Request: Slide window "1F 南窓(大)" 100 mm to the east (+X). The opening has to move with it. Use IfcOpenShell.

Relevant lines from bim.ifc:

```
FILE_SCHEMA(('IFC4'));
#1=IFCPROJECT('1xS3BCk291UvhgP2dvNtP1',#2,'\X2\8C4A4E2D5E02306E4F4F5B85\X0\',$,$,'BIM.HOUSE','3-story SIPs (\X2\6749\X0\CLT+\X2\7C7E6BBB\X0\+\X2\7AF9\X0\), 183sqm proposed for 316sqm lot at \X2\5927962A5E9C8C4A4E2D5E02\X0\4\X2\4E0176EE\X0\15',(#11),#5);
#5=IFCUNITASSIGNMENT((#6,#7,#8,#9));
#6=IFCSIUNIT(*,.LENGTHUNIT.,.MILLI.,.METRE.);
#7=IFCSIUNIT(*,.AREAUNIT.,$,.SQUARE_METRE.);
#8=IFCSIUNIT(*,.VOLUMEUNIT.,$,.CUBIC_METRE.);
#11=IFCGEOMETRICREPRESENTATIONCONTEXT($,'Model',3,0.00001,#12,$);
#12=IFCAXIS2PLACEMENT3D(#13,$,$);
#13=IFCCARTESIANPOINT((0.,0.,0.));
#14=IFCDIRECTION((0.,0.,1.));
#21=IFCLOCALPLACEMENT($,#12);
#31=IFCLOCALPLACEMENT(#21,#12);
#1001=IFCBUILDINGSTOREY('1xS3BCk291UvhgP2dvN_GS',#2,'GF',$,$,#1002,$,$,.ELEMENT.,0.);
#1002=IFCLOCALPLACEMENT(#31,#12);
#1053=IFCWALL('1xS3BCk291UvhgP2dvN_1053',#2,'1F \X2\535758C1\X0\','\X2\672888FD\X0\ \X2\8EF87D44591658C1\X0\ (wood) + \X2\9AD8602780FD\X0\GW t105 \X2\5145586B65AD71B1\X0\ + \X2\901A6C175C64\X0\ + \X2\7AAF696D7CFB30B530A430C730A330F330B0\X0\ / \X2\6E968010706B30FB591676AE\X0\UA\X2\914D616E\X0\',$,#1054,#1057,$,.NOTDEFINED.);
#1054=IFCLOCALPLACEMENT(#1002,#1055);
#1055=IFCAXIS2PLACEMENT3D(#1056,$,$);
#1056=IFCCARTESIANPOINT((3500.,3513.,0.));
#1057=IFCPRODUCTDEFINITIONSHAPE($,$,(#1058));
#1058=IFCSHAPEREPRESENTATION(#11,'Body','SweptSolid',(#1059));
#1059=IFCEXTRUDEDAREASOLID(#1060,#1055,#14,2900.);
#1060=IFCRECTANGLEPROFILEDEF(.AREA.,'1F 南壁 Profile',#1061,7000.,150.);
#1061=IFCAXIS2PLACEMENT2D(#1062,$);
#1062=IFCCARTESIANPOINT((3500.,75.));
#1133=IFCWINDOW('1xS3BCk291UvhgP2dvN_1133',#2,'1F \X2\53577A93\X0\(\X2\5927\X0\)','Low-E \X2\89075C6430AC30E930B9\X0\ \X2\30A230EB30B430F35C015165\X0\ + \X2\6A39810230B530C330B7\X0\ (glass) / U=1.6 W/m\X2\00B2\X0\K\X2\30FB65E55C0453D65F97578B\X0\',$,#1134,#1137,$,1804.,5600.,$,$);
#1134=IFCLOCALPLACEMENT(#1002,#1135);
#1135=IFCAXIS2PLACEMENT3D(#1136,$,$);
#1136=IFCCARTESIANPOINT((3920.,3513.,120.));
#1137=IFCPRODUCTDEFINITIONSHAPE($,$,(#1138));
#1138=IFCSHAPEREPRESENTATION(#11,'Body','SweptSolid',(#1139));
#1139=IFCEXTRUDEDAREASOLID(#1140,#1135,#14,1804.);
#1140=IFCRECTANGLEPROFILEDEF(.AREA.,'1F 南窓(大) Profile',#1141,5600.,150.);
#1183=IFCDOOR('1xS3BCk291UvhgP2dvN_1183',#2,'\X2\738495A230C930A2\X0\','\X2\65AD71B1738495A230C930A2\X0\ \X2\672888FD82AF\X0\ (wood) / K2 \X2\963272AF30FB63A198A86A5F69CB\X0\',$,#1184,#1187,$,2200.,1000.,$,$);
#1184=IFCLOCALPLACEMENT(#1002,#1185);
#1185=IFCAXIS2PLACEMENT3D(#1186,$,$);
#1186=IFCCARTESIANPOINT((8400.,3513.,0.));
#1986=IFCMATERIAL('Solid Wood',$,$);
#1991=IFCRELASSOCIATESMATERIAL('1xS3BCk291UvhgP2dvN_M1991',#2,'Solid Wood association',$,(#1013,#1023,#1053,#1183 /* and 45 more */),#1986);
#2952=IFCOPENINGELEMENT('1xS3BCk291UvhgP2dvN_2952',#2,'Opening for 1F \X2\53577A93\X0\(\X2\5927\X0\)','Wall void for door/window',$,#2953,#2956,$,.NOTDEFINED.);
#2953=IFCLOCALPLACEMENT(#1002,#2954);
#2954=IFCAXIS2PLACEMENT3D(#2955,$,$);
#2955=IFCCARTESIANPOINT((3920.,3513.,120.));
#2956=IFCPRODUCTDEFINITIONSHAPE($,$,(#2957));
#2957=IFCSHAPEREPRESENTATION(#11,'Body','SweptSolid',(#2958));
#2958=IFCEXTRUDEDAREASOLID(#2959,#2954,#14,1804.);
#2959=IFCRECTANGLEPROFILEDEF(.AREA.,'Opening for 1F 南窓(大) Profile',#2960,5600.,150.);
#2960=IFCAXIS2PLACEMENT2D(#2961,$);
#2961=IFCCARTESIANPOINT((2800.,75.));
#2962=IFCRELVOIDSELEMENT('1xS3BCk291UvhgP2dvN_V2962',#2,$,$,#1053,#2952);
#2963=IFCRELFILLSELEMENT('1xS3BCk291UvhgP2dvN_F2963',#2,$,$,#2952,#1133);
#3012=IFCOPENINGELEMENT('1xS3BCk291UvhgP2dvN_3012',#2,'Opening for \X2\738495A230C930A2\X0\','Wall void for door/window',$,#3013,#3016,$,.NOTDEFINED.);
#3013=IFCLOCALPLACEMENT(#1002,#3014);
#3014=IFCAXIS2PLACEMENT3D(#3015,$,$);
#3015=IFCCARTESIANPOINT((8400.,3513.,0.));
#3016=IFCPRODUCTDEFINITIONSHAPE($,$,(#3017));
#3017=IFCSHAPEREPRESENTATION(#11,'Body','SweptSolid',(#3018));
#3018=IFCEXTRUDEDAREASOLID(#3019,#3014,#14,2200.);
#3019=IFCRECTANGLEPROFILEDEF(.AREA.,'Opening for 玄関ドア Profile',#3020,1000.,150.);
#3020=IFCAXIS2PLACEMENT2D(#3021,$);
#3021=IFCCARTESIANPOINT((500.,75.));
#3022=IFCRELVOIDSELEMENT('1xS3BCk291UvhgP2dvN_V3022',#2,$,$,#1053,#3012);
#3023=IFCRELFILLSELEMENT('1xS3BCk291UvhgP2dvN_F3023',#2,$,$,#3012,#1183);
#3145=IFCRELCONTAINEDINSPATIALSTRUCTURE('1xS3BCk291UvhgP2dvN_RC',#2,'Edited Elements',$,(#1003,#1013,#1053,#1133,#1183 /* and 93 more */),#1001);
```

```python
import ifcopenshell
import ifcopenshell.api.geometry
import ifcopenshell.util.placement
import ifcopenshell.util.unit

model = ifcopenshell.open("bim.ifc")
unit_scale = ifcopenshell.util.unit.calculate_unit_scale(model)

window = model.by_guid("1xS3BCk291UvhgP2dvN_1133")
opening = window.FillsVoids[0].RelatingOpeningElement
wall = opening.VoidsElements[0].RelatingBuildingElement

wall_matrix = ifcopenshell.util.placement.get_local_placement(wall.ObjectPlacement)
shift = wall_matrix[:3, 0] * 0.1 / unit_scale
before = ifcopenshell.util.placement.get_local_placement(window.ObjectPlacement)[:3, 3].copy()

# The window is not placed relative to its opening, so move both.
for product in (opening, window):
    matrix = ifcopenshell.util.placement.get_local_placement(product.ObjectPlacement)
    matrix[:3, 3] += shift
    ifcopenshell.api.geometry.edit_object_placement(model, product=product, matrix=matrix, is_si=False)

after = ifcopenshell.util.placement.get_local_placement(window.ObjectPlacement)[:3, 3]
print("window moved by", (after - before).round(3) + 0.0)

model.write("bim_updated.ifc")
```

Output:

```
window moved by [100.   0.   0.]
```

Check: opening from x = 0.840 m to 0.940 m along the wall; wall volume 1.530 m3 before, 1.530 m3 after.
